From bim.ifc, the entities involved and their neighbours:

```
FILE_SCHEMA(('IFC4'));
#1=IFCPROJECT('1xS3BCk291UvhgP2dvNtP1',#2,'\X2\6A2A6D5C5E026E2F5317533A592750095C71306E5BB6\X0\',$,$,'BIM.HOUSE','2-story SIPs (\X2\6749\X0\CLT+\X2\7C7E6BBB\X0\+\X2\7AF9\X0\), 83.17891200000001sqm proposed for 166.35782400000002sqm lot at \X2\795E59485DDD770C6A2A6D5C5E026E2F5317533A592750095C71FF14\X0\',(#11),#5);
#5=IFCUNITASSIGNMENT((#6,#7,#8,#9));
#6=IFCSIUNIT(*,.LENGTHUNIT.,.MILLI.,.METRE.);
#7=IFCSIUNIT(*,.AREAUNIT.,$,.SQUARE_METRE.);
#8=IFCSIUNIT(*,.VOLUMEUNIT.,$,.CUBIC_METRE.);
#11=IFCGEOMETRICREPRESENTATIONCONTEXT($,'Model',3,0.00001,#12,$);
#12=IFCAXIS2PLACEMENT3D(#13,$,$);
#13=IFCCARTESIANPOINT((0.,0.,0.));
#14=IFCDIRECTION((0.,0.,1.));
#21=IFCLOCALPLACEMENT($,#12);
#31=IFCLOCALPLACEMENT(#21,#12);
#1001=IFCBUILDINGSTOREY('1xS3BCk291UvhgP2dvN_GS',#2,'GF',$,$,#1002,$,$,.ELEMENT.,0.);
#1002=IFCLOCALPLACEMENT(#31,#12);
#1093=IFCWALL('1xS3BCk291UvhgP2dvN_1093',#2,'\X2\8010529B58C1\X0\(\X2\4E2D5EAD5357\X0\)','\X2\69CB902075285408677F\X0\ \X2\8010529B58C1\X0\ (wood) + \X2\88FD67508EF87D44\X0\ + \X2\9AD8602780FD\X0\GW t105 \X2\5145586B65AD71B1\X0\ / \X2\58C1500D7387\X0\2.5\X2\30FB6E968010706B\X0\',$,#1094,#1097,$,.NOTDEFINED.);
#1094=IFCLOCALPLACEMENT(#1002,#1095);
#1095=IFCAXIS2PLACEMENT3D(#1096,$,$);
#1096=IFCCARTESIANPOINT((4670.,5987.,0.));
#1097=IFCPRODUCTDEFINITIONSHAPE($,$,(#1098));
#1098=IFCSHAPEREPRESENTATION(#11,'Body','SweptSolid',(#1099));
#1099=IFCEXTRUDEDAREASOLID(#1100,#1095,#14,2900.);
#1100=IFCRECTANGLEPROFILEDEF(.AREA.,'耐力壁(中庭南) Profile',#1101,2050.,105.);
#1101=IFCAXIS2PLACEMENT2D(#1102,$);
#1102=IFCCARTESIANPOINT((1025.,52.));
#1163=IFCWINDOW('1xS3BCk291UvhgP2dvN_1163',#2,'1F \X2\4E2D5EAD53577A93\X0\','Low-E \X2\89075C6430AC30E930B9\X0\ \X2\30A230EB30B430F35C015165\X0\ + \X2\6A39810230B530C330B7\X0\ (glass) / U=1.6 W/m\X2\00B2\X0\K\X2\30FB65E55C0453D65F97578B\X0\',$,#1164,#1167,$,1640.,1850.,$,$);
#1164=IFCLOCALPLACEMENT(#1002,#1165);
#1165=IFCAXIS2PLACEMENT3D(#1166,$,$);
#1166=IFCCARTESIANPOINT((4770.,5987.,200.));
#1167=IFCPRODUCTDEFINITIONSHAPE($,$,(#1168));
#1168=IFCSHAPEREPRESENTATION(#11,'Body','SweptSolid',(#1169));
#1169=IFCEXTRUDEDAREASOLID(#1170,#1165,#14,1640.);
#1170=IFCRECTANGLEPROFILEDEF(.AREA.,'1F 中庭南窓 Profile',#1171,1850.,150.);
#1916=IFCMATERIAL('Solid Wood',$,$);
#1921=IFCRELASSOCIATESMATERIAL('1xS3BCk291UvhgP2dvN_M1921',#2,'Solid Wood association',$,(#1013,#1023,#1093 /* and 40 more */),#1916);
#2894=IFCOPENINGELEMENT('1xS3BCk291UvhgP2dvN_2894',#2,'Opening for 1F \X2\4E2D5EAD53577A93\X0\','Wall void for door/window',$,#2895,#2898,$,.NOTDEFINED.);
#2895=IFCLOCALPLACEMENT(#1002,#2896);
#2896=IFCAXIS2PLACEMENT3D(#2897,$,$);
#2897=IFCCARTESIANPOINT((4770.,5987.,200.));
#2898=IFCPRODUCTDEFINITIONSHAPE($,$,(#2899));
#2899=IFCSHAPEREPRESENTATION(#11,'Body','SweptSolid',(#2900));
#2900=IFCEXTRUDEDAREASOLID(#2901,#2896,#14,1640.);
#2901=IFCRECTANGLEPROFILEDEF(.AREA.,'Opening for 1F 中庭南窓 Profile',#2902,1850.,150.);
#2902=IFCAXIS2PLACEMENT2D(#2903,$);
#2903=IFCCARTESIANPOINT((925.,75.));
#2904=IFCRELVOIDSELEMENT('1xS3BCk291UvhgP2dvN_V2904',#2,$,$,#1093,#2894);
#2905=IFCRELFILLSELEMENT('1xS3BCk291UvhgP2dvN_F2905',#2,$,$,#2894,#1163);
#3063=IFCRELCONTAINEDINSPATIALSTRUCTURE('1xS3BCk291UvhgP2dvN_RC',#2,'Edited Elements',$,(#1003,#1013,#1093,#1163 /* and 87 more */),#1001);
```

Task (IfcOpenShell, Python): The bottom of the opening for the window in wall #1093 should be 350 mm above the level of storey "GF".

```python
import numpy as np
import ifcopenshell
import ifcopenshell.api.geometry
import ifcopenshell.geom
import ifcopenshell.util.element
import ifcopenshell.util.placement
import ifcopenshell.util.shape
import ifcopenshell.util.unit

model = ifcopenshell.open("bim.ifc")
unit_scale = ifcopenshell.util.unit.calculate_unit_scale(model)

window = model.by_guid("1xS3BCk291UvhgP2dvN_1163")
opening = window.FillsVoids[0].RelatingOpeningElement
storey = ifcopenshell.util.element.get_container(window, ifc_class="IfcBuildingStorey")
level = ifcopenshell.util.placement.get_local_placement(storey.ObjectPlacement)[2, 3]

# The opening's origin need not be at the sill, so measure its lowest point.
shape = ifcopenshell.geom.create_shape(ifcopenshell.geom.settings(), opening)
bottom = ifcopenshell.util.shape.get_shape_bottom_elevation(shape, shape.geometry) / unit_scale
dz = level + 0.35 / unit_scale - bottom

shift = np.array([0.0, 0.0, dz])
# The window is not placed relative to its opening, so move both.
for product in (opening, window):
    matrix = ifcopenshell.util.placement.get_local_placement(product.ObjectPlacement)
    matrix[:3, 3] += shift
    ifcopenshell.api.geometry.edit_object_placement(model, product=product, matrix=matrix, is_si=False)

print(f"moved by {dz * unit_scale:+.3f} m")

model.write("bim_edited.ifc")
```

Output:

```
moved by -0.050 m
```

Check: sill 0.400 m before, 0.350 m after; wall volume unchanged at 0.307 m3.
